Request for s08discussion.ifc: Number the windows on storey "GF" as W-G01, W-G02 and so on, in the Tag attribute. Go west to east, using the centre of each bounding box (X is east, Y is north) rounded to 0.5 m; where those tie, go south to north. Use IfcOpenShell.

First a look at what the model holds.

```python
import ifcopenshell
import ifcopenshell.util.element
import ifcopenshell.util.placement

model = ifcopenshell.open("s08discussion.ifc")
print(model.schema)
storey = next(s for s in model.by_type("IfcBuildingStorey") if s.Name == "GF")
windows = [e for e in ifcopenshell.util.element.get_decomposition(storey) if e.is_a("IfcWindow")]
for e in sorted(windows, key=lambda e: e.id()):
    origin = ifcopenshell.util.placement.get_local_placement(e.ObjectPlacement)[:3, 3]
    print(e.id(), e.Tag, e.Name, origin.round(2) + 0.0, sep=" | ")
```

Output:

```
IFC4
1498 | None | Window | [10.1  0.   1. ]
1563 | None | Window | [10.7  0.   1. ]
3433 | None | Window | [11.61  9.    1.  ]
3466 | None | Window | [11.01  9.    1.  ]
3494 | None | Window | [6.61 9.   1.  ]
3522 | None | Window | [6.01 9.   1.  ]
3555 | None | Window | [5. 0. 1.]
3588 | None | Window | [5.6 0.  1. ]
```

```python
import ifcopenshell
import ifcopenshell.geom
import ifcopenshell.util.element
import ifcopenshell.util.shape

model = ifcopenshell.open("s08discussion.ifc")
settings = ifcopenshell.geom.settings()
settings.set("use-world-coords", True)


def centre(element):
    shape = ifcopenshell.geom.create_shape(settings, element)
    return ifcopenshell.util.shape.get_bbox_centroid(shape.geometry)


storey = next(s for s in model.by_type("IfcBuildingStorey") if s.Name == "GF")
windows = [e for e in ifcopenshell.util.element.get_decomposition(storey) if e.is_a("IfcWindow")]

# Insertion points can sit at a corner or the storey origin, so sort by the geometry (in metres).
centres = {e: centre(e) for e in windows}
windows.sort(key=lambda e: (round(centres[e][0] / 0.5), centres[e][1]))

for i, e in enumerate(windows, start=1):
    number = f"W-G{i:02d}"
    e.Tag = number
    print(e.id(), number)

model.write("s08discussion_updated.ifc")
```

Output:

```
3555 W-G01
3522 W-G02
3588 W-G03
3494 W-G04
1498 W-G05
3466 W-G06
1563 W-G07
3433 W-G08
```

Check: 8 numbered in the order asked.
